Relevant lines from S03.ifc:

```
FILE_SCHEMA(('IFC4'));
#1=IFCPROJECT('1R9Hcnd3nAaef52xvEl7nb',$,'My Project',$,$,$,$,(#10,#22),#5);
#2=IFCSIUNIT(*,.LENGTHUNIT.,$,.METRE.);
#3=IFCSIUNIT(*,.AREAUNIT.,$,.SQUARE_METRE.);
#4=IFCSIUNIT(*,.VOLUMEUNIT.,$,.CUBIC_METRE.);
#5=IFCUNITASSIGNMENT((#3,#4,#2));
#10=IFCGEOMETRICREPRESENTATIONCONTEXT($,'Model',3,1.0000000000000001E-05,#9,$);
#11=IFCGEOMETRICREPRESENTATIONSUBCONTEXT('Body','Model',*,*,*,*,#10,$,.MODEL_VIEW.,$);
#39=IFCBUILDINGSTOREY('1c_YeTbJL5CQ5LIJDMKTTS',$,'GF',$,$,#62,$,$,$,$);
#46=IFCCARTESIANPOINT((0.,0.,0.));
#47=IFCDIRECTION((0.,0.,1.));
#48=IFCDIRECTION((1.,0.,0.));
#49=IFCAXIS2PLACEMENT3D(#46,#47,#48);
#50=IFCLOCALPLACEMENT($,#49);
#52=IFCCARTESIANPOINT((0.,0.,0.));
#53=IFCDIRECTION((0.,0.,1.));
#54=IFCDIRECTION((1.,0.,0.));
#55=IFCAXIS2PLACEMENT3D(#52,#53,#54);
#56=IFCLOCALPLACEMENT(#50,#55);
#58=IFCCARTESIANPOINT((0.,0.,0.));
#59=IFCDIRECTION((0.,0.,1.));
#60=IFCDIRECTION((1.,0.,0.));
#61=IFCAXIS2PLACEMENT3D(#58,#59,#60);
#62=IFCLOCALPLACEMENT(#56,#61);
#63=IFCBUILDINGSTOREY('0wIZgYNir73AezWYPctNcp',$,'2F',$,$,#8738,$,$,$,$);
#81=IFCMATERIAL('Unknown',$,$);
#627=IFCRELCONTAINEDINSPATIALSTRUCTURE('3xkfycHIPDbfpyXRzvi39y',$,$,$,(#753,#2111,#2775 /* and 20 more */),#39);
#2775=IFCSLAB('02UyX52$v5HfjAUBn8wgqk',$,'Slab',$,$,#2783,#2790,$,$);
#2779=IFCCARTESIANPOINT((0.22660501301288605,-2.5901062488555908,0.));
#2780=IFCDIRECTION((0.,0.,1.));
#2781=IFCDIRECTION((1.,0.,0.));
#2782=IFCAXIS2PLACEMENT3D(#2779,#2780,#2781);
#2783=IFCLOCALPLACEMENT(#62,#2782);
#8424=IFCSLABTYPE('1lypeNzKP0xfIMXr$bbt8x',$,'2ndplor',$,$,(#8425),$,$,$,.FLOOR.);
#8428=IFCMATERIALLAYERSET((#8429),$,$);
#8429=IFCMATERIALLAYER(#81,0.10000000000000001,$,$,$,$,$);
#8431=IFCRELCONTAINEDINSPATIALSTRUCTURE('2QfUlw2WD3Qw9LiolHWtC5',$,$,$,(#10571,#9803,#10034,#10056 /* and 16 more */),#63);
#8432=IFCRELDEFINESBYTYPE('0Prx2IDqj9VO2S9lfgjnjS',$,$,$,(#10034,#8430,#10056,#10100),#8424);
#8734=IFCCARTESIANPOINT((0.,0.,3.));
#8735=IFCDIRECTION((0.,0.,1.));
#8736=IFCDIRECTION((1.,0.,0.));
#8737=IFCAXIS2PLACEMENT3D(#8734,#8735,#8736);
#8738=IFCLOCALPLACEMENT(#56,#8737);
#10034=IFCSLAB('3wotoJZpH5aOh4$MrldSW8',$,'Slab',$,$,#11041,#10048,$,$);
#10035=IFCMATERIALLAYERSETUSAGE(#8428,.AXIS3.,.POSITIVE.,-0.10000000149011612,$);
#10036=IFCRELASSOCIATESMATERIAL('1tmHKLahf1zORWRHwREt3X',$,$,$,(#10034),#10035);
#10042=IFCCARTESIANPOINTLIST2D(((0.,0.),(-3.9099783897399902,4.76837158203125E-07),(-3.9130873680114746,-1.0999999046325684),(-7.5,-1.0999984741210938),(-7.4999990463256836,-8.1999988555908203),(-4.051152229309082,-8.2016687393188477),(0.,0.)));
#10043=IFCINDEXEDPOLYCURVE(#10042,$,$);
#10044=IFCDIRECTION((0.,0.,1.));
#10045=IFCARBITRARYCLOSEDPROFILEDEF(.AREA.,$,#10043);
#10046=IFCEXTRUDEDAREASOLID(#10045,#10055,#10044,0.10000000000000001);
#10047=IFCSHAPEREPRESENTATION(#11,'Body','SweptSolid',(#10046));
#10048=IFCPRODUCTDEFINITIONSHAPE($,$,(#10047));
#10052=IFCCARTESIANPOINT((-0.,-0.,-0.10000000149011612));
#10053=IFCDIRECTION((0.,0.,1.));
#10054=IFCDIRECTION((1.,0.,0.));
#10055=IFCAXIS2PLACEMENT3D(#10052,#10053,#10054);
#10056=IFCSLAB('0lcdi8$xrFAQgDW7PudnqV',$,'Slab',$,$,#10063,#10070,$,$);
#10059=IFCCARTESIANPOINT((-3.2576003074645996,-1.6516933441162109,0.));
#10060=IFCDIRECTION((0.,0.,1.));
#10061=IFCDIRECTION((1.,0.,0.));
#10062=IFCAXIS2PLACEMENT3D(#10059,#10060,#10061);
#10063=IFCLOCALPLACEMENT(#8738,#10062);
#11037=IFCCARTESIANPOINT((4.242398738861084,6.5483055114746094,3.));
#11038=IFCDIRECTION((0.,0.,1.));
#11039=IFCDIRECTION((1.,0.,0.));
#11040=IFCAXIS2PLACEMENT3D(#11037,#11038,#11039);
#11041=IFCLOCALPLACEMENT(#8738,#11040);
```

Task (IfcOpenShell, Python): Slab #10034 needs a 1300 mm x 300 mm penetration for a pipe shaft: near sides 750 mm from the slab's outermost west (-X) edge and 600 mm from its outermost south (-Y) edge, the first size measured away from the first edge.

```python
import numpy as np
import ifcopenshell
import ifcopenshell.api.feature
import ifcopenshell.api.geometry
import ifcopenshell.api.root
import ifcopenshell.geom
import ifcopenshell.util.placement
import ifcopenshell.util.representation
import ifcopenshell.util.shape
import ifcopenshell.util.unit

model = ifcopenshell.open("S03.ifc")
unit_scale = ifcopenshell.util.unit.calculate_unit_scale(model)
settings = ifcopenshell.geom.settings()


def volume(element):
    """Net volume in cubic metres, openings subtracted."""
    shape = ifcopenshell.geom.create_shape(settings, element)
    return ifcopenshell.util.shape.get_volume(shape.geometry)


slab = model.by_guid("3wotoJZpH5aOh4$MrldSW8")
before = volume(slab)

# Extent in the slab's own axes, in metres. The edges named are its -X and -Y sides.
slab_shape = ifcopenshell.geom.create_shape(settings, slab)
vertices = ifcopenshell.util.shape.get_vertices(slab_shape.geometry)
x_min, y_min, bottom = vertices.min(axis=0)
top = vertices[:, 2].max()

opening = ifcopenshell.api.root.create_entity(model, ifc_class="IfcOpeningElement", name="Pipe shaft opening", predefined_type="OPENING")
context = ifcopenshell.util.representation.get_context(model, "Model", "Body", "MODEL_VIEW")
width, depth = 1.3, 0.3
outline = [(0.0, 0.0), (width, 0.0), (width, depth), (0.0, depth), (0.0, 0.0)]
# Overshoot both faces by 50 mm so the cut is clean.
shape = ifcopenshell.api.geometry.add_slab_representation(
    model, context=context, depth=top - bottom + 0.1, polyline=outline
)
ifcopenshell.api.geometry.assign_representation(model, product=opening, representation=shape)

matrix = ifcopenshell.util.placement.get_local_placement(slab.ObjectPlacement)
matrix[:, 3] = matrix @ np.append(np.array([x_min + 0.75, y_min + 0.6, bottom - 0.05]) / unit_scale, 1.0)
ifcopenshell.api.geometry.edit_object_placement(model, product=opening, matrix=matrix, is_si=False)
ifcopenshell.api.feature.add_feature(model, feature=opening, element=slab)

after = volume(slab)

print(f"slab volume {before:.3f} -> {after:.3f} m3")

model.write("S03_rev.ifc")
```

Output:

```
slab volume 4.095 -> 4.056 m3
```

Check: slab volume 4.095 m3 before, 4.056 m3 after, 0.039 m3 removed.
